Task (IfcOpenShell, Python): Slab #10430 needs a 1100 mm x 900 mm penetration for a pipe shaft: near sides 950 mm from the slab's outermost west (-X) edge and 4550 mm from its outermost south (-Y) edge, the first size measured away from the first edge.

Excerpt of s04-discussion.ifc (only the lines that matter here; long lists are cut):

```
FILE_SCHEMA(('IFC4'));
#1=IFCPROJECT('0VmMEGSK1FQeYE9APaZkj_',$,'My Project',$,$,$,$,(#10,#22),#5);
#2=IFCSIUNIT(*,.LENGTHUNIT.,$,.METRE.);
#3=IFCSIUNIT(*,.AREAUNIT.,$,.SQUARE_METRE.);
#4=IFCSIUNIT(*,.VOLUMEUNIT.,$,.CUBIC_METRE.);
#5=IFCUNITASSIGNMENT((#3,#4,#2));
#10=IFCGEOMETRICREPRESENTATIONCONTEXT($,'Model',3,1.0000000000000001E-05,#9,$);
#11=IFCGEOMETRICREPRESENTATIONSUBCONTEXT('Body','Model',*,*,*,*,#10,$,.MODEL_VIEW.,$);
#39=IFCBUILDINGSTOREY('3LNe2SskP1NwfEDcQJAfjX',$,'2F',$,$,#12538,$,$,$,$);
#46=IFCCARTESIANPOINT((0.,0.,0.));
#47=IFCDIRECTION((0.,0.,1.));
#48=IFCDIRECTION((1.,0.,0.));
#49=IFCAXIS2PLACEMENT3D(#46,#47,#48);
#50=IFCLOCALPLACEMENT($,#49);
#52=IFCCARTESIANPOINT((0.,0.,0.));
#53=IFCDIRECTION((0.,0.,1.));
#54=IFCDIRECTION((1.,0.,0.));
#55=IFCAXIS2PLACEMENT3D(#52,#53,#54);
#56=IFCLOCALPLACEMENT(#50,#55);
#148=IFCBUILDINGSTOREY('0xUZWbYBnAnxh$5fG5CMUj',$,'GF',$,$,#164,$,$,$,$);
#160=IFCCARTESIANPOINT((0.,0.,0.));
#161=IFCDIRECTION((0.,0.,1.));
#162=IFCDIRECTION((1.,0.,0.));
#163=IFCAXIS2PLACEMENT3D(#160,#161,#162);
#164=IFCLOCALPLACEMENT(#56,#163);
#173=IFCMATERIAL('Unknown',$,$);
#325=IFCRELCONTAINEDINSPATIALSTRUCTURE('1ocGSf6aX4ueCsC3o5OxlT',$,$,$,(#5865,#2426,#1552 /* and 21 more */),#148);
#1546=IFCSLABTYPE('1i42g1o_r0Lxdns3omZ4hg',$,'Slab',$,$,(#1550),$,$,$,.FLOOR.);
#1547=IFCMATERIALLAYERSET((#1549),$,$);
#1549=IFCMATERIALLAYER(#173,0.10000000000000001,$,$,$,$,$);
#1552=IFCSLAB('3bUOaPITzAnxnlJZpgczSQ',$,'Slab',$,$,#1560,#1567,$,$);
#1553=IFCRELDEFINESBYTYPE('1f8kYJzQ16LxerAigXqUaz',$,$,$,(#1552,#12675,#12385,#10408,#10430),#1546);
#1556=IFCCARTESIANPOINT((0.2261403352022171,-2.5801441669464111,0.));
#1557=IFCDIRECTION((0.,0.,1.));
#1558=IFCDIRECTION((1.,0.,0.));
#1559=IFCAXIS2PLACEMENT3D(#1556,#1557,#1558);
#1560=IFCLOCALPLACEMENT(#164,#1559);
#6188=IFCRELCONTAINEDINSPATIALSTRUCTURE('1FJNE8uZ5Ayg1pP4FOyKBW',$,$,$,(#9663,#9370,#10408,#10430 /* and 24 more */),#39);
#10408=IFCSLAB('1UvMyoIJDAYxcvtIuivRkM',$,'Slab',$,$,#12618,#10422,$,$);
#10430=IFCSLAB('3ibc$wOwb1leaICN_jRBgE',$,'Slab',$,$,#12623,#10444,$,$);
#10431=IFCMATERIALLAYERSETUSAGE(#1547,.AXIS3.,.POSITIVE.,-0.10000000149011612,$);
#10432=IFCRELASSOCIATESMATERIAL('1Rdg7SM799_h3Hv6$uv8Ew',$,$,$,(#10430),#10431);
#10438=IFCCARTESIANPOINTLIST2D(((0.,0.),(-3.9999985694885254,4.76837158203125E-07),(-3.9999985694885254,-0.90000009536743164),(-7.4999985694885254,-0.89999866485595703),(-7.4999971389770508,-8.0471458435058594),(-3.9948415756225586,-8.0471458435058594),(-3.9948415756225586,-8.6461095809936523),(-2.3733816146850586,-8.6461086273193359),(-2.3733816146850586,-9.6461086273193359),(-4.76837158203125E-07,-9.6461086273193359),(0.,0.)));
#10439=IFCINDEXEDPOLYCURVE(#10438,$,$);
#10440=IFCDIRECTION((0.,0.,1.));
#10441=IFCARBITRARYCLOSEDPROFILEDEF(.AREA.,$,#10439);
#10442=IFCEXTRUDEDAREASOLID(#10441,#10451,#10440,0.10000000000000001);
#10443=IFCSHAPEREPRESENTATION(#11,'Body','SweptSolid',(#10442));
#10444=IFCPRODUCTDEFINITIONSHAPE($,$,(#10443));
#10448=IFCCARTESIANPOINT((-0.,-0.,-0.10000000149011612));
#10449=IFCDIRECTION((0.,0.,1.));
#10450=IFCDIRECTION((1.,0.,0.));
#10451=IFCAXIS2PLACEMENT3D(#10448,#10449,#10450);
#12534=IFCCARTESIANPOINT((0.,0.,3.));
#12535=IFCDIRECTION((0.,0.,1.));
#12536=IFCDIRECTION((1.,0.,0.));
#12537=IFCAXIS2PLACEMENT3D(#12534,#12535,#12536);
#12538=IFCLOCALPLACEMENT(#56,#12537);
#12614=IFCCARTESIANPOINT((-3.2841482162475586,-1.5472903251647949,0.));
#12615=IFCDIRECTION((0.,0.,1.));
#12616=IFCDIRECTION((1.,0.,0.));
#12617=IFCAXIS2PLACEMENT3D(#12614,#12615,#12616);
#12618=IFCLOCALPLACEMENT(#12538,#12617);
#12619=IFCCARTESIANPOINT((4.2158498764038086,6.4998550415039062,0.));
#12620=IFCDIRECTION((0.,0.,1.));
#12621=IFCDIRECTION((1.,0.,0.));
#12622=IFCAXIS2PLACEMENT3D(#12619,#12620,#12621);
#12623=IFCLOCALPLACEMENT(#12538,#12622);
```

```python
import numpy as np
import ifcopenshell
import ifcopenshell.api.feature
import ifcopenshell.api.geometry
import ifcopenshell.api.root
import ifcopenshell.geom
import ifcopenshell.util.placement
import ifcopenshell.util.representation
import ifcopenshell.util.shape
import ifcopenshell.util.unit

model = ifcopenshell.open("s04-discussion.ifc")
unit_scale = ifcopenshell.util.unit.calculate_unit_scale(model)
settings = ifcopenshell.geom.settings()


def volume(element):
    """Net volume in cubic metres, openings subtracted."""
    shape = ifcopenshell.geom.create_shape(settings, element)
    return ifcopenshell.util.shape.get_volume(shape.geometry)


slab = model.by_id(10430)
before = volume(slab)

# Extent in the slab's own axes, in metres. The edges named are its -X and -Y sides.
slab_shape = ifcopenshell.geom.create_shape(settings, slab)
vertices = ifcopenshell.util.shape.get_vertices(slab_shape.geometry)
x_min, y_min, bottom = vertices.min(axis=0)
top = vertices[:, 2].max()

opening = ifcopenshell.api.root.create_entity(model, ifc_class="IfcOpeningElement", name="Pipe shaft opening", predefined_type="OPENING")
context = ifcopenshell.util.representation.get_context(model, "Model", "Body", "MODEL_VIEW")
width, depth = 1.1, 0.9
outline = [(0.0, 0.0), (width, 0.0), (width, depth), (0.0, depth), (0.0, 0.0)]
# Overshoot both faces by 50 mm so the cut is clean.
shape = ifcopenshell.api.geometry.add_slab_representation(
    model, context=context, depth=top - bottom + 0.1, polyline=outline
)
ifcopenshell.api.geometry.assign_representation(model, product=opening, representation=shape)

matrix = ifcopenshell.util.placement.get_local_placement(slab.ObjectPlacement)
matrix[:, 3] = matrix @ np.append(np.array([x_min + 0.95, y_min + 4.55, bottom - 0.05]) / unit_scale, 1.0)
ifcopenshell.api.geometry.edit_object_placement(model, product=opening, matrix=matrix, is_si=False)
ifcopenshell.api.feature.add_feature(model, feature=opening, element=slab)

after = volume(slab)

print(f"slab volume {before:.3f} -> {after:.3f} m3")

model.write("s04-discussion-out.ifc")
```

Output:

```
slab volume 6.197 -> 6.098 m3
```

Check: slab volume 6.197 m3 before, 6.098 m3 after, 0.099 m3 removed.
